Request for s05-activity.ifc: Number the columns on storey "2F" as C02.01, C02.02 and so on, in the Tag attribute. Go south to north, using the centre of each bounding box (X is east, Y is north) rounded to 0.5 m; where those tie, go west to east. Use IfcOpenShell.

First a look at what the model holds.

```python
import ifcopenshell
import ifcopenshell.util.element
import ifcopenshell.util.placement

model = ifcopenshell.open("s05-activity.ifc")
print(model.schema)
storey = next(s for s in model.by_type("IfcBuildingStorey") if s.Name == "2F")
columns = [e for e in ifcopenshell.util.element.get_decomposition(storey) if e.is_a("IfcColumn")]
for e in sorted(columns, key=lambda e: e.id()):
    origin = ifcopenshell.util.placement.get_local_placement(e.ObjectPlacement)[:3, 3]
    print(e.id(), e.Tag, e.Name, origin.round(2) + 0.0, sep=" | ")
```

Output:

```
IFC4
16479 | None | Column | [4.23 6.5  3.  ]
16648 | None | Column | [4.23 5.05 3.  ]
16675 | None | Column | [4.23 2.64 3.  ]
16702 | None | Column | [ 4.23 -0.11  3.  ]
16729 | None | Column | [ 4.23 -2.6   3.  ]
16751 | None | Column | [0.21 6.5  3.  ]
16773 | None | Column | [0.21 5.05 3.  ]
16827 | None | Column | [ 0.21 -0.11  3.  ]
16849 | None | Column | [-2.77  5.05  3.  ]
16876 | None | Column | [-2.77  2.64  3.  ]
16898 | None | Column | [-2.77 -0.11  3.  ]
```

```python
import ifcopenshell
import ifcopenshell.geom
import ifcopenshell.util.element
import ifcopenshell.util.shape

model = ifcopenshell.open("s05-activity.ifc")
settings = ifcopenshell.geom.settings()
settings.set("use-world-coords", True)


def centre(element):
    shape = ifcopenshell.geom.create_shape(settings, element)
    return ifcopenshell.util.shape.get_bbox_centroid(shape.geometry)


storey = next(s for s in model.by_type("IfcBuildingStorey") if s.Name == "2F")
columns = [e for e in ifcopenshell.util.element.get_decomposition(storey) if e.is_a("IfcColumn")]

# Insertion points can sit at a corner or the storey origin, so sort by the geometry (in metres).
centres = {e: centre(e) for e in columns}
columns.sort(key=lambda e: (round(centres[e][1] / 0.5), centres[e][0]))

for i, e in enumerate(columns, start=1):
    number = f"C02.{i:02d}"
    e.Tag = number
    print(e.id(), number)

model.write("s05-activity_edited.ifc")
```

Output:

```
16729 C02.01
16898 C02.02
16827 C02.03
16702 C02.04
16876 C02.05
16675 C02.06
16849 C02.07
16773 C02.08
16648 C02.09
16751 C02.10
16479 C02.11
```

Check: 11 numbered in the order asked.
